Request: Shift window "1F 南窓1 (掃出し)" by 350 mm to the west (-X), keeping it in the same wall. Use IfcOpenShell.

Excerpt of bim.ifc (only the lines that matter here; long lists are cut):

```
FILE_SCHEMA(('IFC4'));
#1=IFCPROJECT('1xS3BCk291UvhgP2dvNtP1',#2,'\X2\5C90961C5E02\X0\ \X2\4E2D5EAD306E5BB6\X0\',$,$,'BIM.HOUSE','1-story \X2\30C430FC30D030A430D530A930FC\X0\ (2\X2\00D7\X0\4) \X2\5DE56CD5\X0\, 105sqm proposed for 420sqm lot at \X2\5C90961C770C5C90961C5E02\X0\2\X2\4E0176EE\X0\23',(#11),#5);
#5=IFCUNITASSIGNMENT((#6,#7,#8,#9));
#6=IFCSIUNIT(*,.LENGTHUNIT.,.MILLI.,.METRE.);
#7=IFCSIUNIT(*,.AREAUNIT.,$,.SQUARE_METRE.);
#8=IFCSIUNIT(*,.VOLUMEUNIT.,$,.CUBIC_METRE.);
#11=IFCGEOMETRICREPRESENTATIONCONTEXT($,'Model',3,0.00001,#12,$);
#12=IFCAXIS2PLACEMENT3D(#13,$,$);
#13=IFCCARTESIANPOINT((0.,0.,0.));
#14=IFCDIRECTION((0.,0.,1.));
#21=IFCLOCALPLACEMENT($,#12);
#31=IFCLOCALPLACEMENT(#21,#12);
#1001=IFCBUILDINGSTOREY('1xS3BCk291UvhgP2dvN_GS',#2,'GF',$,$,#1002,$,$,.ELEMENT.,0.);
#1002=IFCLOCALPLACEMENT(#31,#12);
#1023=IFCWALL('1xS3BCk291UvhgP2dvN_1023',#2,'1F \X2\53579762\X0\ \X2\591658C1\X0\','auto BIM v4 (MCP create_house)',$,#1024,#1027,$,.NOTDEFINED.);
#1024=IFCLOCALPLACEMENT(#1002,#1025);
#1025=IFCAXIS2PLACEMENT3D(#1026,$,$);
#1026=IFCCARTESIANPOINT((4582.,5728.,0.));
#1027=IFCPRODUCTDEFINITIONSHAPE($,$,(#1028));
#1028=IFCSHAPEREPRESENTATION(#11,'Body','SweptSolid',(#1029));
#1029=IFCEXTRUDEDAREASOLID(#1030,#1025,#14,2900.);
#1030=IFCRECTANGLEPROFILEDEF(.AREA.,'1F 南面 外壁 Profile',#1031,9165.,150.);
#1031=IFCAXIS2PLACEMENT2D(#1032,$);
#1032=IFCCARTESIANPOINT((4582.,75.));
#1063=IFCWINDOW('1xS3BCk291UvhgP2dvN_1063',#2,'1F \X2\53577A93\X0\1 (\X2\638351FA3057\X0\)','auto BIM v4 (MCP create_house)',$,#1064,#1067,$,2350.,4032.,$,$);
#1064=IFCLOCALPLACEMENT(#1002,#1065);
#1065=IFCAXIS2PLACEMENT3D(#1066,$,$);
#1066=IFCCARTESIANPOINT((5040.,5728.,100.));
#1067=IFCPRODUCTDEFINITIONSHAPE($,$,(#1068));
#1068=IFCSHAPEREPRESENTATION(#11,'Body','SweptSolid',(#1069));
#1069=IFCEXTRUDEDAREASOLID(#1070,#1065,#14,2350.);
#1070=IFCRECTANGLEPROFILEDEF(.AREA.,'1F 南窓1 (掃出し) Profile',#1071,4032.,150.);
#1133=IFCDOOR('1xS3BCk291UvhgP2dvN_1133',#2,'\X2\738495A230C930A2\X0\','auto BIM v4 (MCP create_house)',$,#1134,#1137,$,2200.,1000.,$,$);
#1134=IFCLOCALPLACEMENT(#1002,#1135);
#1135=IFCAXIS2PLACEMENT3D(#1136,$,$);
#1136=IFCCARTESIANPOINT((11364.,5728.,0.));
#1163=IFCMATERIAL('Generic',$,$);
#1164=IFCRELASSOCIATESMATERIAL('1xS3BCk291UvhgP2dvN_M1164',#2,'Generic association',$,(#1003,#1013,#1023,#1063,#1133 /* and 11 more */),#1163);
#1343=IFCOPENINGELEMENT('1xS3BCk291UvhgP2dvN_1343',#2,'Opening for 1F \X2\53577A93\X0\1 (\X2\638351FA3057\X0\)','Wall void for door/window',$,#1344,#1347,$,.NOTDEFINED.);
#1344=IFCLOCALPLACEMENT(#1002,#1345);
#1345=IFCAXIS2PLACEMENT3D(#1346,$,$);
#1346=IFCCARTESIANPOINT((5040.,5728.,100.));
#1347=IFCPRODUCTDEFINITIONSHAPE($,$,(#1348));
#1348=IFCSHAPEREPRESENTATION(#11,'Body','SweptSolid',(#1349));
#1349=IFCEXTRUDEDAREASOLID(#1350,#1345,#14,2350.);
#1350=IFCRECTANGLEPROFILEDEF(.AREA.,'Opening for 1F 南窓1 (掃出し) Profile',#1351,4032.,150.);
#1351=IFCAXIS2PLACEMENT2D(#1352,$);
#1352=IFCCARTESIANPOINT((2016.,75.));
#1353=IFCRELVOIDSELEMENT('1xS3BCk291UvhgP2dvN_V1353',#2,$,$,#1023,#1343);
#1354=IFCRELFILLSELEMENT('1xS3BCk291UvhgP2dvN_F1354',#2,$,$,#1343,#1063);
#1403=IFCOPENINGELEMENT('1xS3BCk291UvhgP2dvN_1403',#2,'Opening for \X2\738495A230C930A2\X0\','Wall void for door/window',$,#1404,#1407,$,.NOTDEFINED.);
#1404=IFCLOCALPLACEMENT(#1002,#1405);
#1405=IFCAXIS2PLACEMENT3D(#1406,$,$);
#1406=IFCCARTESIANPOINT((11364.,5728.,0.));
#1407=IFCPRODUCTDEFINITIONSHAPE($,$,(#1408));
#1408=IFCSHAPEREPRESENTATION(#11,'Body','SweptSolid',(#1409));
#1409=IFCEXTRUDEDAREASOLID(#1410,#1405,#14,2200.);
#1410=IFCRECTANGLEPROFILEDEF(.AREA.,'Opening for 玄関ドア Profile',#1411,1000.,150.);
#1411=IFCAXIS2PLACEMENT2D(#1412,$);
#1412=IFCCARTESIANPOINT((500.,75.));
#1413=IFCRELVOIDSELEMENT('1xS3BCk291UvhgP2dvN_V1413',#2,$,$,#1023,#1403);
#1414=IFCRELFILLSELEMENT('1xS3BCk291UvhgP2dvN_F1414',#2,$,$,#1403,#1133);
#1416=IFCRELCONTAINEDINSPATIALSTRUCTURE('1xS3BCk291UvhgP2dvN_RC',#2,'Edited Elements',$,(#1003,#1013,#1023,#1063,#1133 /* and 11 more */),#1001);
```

```python
import ifcopenshell
import ifcopenshell.api.geometry
import ifcopenshell.util.placement
import ifcopenshell.util.unit

model = ifcopenshell.open("bim.ifc")
unit_scale = ifcopenshell.util.unit.calculate_unit_scale(model)

window = model.by_id(1063)
opening = window.FillsVoids[0].RelatingOpeningElement
wall = opening.VoidsElements[0].RelatingBuildingElement

wall_matrix = ifcopenshell.util.placement.get_local_placement(wall.ObjectPlacement)
shift = wall_matrix[:3, 0] * -0.35 / unit_scale
before = ifcopenshell.util.placement.get_local_placement(window.ObjectPlacement)[:3, 3].copy()

# The window is not placed relative to its opening, so move both.
for product in (opening, window):
    matrix = ifcopenshell.util.placement.get_local_placement(product.ObjectPlacement)
    matrix[:3, 3] += shift
    ifcopenshell.api.geometry.edit_object_placement(model, product=product, matrix=matrix, is_si=False)

after = ifcopenshell.util.placement.get_local_placement(window.ObjectPlacement)[:3, 3]
print("window moved by", (after - before).round(3) + 0.0)

model.write("bim-out.ifc")
```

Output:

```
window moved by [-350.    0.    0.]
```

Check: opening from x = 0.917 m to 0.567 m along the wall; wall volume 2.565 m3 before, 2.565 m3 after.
